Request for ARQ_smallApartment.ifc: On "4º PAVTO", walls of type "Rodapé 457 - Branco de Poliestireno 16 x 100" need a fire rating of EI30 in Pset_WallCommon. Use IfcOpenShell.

First a look at what the model holds.

```python
import ifcopenshell
import ifcopenshell.util.element

model = ifcopenshell.open("ARQ_smallApartment.ifc")
print(model.schema)
storey = next(s for s in model.by_type("IfcBuildingStorey") if s.Name == "4º PAVTO")
walls = [e for e in ifcopenshell.util.element.get_decomposition(storey) if e.is_a("IfcWall")]
seen = {}
for e in walls:
    element_type = ifcopenshell.util.element.get_type(e)
    key = (element_type.Name if element_type != e and element_type else None, ifcopenshell.util.element.get_pset(e, "Pset_WallCommon", "FireRating"))
    seen[key] = seen.get(key, 0) + 1
for (name, value), count in sorted(seen.items(), key=str):
    print(count, "x", name, "|", value)
```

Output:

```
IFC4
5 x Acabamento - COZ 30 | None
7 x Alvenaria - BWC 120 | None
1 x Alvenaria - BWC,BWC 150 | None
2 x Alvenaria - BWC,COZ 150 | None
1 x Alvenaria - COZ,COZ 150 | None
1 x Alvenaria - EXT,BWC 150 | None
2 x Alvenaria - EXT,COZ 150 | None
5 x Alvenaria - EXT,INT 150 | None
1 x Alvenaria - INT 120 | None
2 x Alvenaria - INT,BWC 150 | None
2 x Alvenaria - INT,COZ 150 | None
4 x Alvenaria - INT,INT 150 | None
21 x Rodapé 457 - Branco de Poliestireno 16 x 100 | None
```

```python
import ifcopenshell
import ifcopenshell.api.pset
import ifcopenshell.util.element

model = ifcopenshell.open("ARQ_smallApartment.ifc")

storey = next(s for s in model.by_type("IfcBuildingStorey") if s.Name == "4º PAVTO")
walls = [e for e in ifcopenshell.util.element.get_decomposition(storey) if e.is_a("IfcWall")]

count = 0
for e in walls:
    element_type = ifcopenshell.util.element.get_type(e)
    if element_type in (None, e) or element_type.Name != "Rodapé 457 - Branco de Poliestireno 16 x 100":
        continue
    # add_pset returns the element's existing set when there is one.
    pset = ifcopenshell.api.pset.add_pset(model, product=e, name="Pset_WallCommon")
    ifcopenshell.api.pset.edit_pset(model, pset=pset, properties={"FireRating": "EI30"})
    count += 1

print(count, "walls updated")

model.write("ARQ_smallApartment_edited.ifc")
```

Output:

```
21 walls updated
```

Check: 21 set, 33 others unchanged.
